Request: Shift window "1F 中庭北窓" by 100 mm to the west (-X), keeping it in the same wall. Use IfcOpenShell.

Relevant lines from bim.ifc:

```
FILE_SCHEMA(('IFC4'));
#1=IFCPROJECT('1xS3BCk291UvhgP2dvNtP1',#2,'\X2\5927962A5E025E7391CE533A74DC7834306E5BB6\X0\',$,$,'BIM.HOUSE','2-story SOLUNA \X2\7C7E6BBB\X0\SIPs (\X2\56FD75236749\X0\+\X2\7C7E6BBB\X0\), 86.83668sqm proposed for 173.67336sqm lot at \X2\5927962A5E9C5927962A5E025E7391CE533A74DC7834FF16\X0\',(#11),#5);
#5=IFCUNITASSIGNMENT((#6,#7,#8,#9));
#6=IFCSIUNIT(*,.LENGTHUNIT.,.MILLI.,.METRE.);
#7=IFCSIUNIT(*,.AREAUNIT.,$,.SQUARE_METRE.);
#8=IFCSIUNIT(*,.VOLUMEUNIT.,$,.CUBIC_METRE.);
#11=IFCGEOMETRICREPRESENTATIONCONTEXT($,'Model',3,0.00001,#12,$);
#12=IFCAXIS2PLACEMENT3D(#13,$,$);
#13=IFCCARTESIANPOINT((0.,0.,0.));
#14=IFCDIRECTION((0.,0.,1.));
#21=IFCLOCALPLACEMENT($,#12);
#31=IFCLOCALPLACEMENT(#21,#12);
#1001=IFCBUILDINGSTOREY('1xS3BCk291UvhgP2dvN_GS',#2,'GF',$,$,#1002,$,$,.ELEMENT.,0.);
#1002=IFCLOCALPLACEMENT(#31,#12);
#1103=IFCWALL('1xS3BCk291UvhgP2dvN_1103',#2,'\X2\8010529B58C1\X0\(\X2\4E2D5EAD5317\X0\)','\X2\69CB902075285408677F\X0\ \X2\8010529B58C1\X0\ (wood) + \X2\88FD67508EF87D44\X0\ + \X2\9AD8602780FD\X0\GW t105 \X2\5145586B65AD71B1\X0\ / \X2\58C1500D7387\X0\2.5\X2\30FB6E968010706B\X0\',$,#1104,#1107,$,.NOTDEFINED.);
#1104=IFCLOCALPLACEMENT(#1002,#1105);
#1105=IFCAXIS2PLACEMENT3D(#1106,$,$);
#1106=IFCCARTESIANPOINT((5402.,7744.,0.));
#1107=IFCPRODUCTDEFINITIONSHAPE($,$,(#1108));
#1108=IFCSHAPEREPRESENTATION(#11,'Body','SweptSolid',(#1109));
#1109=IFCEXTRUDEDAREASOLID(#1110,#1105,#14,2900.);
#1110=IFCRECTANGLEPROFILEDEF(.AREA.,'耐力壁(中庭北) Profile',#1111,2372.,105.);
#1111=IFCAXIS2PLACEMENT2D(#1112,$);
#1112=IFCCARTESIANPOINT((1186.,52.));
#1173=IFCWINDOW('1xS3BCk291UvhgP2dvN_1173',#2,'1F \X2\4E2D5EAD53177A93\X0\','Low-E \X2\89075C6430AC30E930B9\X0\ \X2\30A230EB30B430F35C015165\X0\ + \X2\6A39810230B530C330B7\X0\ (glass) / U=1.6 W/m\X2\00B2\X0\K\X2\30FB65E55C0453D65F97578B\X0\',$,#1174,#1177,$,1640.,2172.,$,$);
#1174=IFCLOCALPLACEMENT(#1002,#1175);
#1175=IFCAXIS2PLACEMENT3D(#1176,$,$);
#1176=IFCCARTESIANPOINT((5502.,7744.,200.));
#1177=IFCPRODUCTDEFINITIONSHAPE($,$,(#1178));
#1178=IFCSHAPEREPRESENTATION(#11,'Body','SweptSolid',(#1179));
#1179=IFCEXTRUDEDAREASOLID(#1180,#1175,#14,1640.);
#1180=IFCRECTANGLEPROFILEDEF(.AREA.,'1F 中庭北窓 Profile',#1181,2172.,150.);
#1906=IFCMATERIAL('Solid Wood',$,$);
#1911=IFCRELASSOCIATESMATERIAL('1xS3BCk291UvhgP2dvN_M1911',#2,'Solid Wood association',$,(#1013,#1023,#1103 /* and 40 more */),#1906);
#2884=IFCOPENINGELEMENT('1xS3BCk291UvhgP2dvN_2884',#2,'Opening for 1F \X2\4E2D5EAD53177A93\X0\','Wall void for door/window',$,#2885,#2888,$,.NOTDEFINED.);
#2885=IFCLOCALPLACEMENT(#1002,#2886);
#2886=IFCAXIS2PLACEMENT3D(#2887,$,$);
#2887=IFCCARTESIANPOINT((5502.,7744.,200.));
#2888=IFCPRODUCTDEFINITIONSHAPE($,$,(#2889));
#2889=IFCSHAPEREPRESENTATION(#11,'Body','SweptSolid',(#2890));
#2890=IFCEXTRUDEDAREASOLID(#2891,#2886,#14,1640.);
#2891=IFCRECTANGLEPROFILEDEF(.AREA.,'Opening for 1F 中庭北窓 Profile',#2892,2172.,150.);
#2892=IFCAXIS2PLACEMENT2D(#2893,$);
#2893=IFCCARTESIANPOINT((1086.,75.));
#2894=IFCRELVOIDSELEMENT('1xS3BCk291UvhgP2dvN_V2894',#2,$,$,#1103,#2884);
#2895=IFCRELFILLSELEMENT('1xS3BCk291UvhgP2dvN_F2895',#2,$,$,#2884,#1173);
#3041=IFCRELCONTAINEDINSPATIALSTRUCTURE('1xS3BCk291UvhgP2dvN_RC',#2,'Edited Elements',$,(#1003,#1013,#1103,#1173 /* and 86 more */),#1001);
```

```python
import ifcopenshell
import ifcopenshell.api.geometry
import ifcopenshell.util.placement
import ifcopenshell.util.unit

model = ifcopenshell.open("bim.ifc")
unit_scale = ifcopenshell.util.unit.calculate_unit_scale(model)

window = model.by_guid("1xS3BCk291UvhgP2dvN_1173")
opening = window.FillsVoids[0].RelatingOpeningElement
wall = opening.VoidsElements[0].RelatingBuildingElement

wall_matrix = ifcopenshell.util.placement.get_local_placement(wall.ObjectPlacement)
shift = wall_matrix[:3, 0] * -0.1 / unit_scale
before = ifcopenshell.util.placement.get_local_placement(window.ObjectPlacement)[:3, 3].copy()

# The window is not placed relative to its opening, so move both.
for product in (opening, window):
    matrix = ifcopenshell.util.placement.get_local_placement(product.ObjectPlacement)
    matrix[:3, 3] += shift
    ifcopenshell.api.geometry.edit_object_placement(model, product=product, matrix=matrix, is_si=False)

after = ifcopenshell.util.placement.get_local_placement(window.ObjectPlacement)[:3, 3]
print("window moved by", (after - before).round(3) + 0.0)

model.write("bim_v2.ifc")
```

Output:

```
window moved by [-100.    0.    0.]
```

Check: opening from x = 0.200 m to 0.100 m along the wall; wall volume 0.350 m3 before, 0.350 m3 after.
